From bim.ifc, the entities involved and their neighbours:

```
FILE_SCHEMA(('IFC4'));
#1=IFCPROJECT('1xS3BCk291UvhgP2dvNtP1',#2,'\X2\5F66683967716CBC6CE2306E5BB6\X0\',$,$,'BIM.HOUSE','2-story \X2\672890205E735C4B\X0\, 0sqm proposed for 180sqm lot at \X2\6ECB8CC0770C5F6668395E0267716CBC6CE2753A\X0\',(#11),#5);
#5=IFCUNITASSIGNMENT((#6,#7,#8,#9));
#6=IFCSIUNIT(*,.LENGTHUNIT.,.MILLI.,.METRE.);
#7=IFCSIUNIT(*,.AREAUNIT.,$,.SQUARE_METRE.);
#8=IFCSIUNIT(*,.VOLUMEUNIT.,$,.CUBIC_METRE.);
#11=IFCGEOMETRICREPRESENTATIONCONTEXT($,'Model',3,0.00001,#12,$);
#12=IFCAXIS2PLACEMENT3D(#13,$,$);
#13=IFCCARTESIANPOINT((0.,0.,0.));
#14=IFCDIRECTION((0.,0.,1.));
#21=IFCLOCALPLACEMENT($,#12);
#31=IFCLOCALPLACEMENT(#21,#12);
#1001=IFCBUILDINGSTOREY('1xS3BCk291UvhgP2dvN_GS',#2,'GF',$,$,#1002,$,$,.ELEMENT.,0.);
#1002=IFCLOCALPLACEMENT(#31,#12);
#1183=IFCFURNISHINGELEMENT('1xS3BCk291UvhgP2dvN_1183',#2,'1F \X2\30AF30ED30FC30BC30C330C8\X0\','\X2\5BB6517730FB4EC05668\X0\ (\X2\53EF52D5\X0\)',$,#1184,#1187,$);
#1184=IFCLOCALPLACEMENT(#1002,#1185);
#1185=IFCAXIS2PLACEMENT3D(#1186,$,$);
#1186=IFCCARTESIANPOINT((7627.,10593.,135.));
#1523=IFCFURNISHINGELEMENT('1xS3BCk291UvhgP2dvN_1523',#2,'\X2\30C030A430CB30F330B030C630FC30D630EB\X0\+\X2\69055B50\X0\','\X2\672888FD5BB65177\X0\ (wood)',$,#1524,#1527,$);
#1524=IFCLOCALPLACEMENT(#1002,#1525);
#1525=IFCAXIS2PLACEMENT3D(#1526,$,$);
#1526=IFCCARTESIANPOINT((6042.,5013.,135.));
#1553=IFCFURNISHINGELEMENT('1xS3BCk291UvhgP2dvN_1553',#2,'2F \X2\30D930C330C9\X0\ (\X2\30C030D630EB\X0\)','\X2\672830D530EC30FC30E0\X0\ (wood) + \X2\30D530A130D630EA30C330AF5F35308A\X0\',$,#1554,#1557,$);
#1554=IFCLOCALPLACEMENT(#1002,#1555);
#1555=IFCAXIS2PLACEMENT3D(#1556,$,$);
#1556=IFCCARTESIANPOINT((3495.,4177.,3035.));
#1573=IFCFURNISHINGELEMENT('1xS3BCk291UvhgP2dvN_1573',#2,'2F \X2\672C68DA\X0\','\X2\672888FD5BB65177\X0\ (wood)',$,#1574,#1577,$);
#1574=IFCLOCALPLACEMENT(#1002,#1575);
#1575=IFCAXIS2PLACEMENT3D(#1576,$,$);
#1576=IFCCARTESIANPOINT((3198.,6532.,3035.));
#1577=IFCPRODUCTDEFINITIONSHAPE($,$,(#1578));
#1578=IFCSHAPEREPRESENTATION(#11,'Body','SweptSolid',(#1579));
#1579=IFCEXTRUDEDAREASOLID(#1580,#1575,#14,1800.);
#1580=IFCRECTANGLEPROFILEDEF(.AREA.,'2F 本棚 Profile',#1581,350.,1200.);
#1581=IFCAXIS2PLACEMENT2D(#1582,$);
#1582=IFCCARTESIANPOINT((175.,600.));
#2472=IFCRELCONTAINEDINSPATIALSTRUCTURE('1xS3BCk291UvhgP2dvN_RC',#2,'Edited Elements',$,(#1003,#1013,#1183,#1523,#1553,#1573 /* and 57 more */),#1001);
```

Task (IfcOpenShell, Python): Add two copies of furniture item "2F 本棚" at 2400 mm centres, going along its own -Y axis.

```python
import ifcopenshell
import ifcopenshell.api.geometry
import ifcopenshell.api.root
import ifcopenshell.util.element
import ifcopenshell.util.placement
import ifcopenshell.util.unit

model = ifcopenshell.open("bim.ifc")
unit_scale = ifcopenshell.util.unit.calculate_unit_scale(model)


def reuse_history(source, copy):
    """copy_class also copies each property set's owner history, people and application; keep the originals."""
    for rel in copy.IsDefinedBy:
        if rel.is_a("IfcRelDefinesByProperties") and (history := rel.RelatingPropertyDefinition.OwnerHistory):
            rel.RelatingPropertyDefinition.OwnerHistory = source.OwnerHistory
            ifcopenshell.util.element.remove_deep2(model, history)


source = model.by_guid("1xS3BCk291UvhgP2dvN_1573")
base = ifcopenshell.util.placement.get_local_placement(source.ObjectPlacement)
step = -base[:3, 1] * 2.4 / unit_scale

for i in range(1, 3):
    copy = ifcopenshell.api.root.copy_class(model, product=source)
    copy.Representation = ifcopenshell.util.element.copy_deep(
        model, source.Representation, exclude=["IfcGeometricRepresentationContext", "IfcRepresentationMap"]
    )
    reuse_history(source, copy)
    matrix = base.copy()
    matrix[:3, 3] += i * step
    print("added at", matrix[:3, 3].round(3) + 0.0)
    ifcopenshell.api.geometry.edit_object_placement(model, product=copy, matrix=matrix, is_si=False)

model.write("bim_edited.ifc")
```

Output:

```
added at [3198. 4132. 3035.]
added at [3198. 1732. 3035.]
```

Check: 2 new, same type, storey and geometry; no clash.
